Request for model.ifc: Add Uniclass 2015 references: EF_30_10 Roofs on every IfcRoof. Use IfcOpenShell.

First a look at what the model holds.

```python
import ifcopenshell

model = ifcopenshell.open("model.ifc")
print(model.schema)
print("classifications:", [c.Name for c in model.by_type("IfcClassification")])
for ifc_class in ("IfcDoor", "IfcRoof", "IfcStair", "IfcWall", "IfcWindow"):
    print(ifc_class, len(model.by_type(ifc_class)))
```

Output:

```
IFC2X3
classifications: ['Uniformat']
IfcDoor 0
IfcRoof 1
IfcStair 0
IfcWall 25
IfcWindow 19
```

```python
import ifcopenshell
import ifcopenshell.api.classification

model = ifcopenshell.open("model.ifc")

# IFC2X3 requires Source and Edition and has no link from the project to the system.
system = model.create_entity("IfcClassification", Source="NBS", Edition="2015", Name="Uniclass 2015")

codes = {
    "IfcRoof": ("EF_30_10", "Roofs"),
}
for ifc_class, (code, name) in codes.items():
    products = model.by_type(ifc_class)
    ifcopenshell.api.classification.add_reference(
        model, products=products, classification=system, identification=code, name=name
    )
    print(code, len(products))

model.write("model_v2.ifc")
```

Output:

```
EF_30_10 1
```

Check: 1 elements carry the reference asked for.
